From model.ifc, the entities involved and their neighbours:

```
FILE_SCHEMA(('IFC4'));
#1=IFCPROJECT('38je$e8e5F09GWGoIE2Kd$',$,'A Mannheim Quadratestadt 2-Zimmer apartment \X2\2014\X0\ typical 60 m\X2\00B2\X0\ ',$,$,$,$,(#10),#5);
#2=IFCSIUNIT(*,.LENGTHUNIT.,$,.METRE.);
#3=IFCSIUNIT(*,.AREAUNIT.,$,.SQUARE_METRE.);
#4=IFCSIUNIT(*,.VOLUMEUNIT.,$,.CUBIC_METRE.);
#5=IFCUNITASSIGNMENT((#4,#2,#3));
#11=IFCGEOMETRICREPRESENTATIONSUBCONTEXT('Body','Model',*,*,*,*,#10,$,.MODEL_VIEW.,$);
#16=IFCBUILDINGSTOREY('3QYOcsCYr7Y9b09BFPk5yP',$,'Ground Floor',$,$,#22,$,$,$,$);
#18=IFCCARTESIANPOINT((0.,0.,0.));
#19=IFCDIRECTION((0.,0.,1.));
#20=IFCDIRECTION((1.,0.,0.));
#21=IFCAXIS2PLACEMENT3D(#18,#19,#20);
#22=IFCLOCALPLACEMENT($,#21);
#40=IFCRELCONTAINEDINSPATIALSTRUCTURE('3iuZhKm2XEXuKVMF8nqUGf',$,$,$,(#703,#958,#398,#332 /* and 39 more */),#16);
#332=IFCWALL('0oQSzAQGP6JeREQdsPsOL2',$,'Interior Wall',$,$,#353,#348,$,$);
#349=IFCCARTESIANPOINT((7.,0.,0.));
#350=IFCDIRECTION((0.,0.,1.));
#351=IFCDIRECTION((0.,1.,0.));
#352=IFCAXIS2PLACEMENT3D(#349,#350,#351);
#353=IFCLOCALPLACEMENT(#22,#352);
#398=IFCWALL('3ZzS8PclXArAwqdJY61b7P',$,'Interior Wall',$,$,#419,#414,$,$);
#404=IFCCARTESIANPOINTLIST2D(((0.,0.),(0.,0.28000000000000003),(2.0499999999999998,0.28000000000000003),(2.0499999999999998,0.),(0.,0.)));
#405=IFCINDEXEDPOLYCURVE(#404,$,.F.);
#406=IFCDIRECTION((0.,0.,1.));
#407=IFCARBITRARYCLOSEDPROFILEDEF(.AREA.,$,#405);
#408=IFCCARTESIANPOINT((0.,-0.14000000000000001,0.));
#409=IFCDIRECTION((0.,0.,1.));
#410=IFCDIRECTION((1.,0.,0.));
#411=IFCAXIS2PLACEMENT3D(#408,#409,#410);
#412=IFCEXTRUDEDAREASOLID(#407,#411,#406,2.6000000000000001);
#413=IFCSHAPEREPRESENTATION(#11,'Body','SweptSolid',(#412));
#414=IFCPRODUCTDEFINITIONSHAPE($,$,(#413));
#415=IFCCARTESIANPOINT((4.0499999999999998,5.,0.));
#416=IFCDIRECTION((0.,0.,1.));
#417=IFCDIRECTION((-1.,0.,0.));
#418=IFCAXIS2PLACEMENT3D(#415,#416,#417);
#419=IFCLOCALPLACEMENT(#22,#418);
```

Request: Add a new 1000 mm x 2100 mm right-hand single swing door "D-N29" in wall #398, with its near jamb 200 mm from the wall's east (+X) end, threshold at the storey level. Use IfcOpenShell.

```python
import numpy as np
import ifcopenshell
import ifcopenshell.api.feature
import ifcopenshell.api.geometry
import ifcopenshell.api.root
import ifcopenshell.api.spatial
import ifcopenshell.geom
import ifcopenshell.util.element
import ifcopenshell.util.placement
import ifcopenshell.util.representation
import ifcopenshell.util.shape
import ifcopenshell.util.unit

model = ifcopenshell.open("model.ifc")
unit_scale = ifcopenshell.util.unit.calculate_unit_scale(model)
settings = ifcopenshell.geom.settings()


def volume(element):
    """Net volume in cubic metres, openings subtracted."""
    shape = ifcopenshell.geom.create_shape(settings, element)
    return ifcopenshell.util.shape.get_volume(shape.geometry)


wall = model.by_guid("3ZzS8PclXArAwqdJY61b7P")
storey = ifcopenshell.util.element.get_container(wall, ifc_class="IfcBuildingStorey")
context = ifcopenshell.util.representation.get_context(model, "Model", "Body", "MODEL_VIEW")
before = volume(wall)

width, height, from_end, sill = 1, 2.1, 0.2, 0.0  # metres

# The wall runs along its own X axis, and the end named is its -X end.
wall_shape = ifcopenshell.geom.create_shape(settings, wall)
x, y, z = ifcopenshell.util.shape.get_vertices(wall_shape.geometry).T
start = x.min() + from_end
face, thickness = float(y.min()), float(y.max() - y.min())
wall_matrix = ifcopenshell.util.placement.get_local_placement(wall.ObjectPlacement)
level = ifcopenshell.util.placement.get_local_placement(storey.ObjectPlacement)[2, 3]


def in_wall(x, y):
    """Placement at x, y metres in the wall's axes, at sill height."""
    matrix = wall_matrix.copy()
    matrix[:, 3] = wall_matrix @ np.array([x / unit_scale, y / unit_scale, 0.0, 1.0])
    matrix[2, 3] = level + sill / unit_scale
    return matrix


# Opening: a box that overshoots both wall faces by 50 mm.
opening = ifcopenshell.api.root.create_entity(model, ifc_class="IfcOpeningElement", predefined_type="OPENING")
box = ifcopenshell.api.geometry.add_wall_representation(
    model, context=context, length=width, height=height, thickness=thickness + 0.1
)
ifcopenshell.api.geometry.assign_representation(model, product=opening, representation=box)
ifcopenshell.api.geometry.edit_object_placement(model, product=opening, matrix=in_wall(start, face - 0.05), is_si=False)
ifcopenshell.api.feature.add_feature(model, feature=opening, element=wall)

door = ifcopenshell.api.root.create_entity(model, ifc_class="IfcDoor", name="D-N29", predefined_type="DOOR")
door.OverallWidth, door.OverallHeight = width / unit_scale, height / unit_scale
door.OperationType = "SINGLE_SWING_RIGHT"
body = ifcopenshell.api.geometry.add_door_representation(
    model,
    context=context,
    overall_width=door.OverallWidth,
    overall_height=door.OverallHeight,
    operation_type="SINGLE_SWING_RIGHT",
    lining_properties={"LiningDepth": thickness / unit_scale, "ThresholdDepth": thickness / unit_scale},
)
ifcopenshell.api.geometry.assign_representation(model, product=door, representation=body)
ifcopenshell.api.spatial.assign_container(model, products=[door], relating_structure=storey)
ifcopenshell.api.feature.add_filling(model, opening=opening, element=door)

# The lining spans the wall, so the door starts at the wall face.
ifcopenshell.api.geometry.edit_object_placement(model, product=door, matrix=in_wall(start, face), is_si=False)

after = volume(wall)

print(f"wall volume {before:.3f} -> {after:.3f} m3")

model.write("model_v2.ifc")
```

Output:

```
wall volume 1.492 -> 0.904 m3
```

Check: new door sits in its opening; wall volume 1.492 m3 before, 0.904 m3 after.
